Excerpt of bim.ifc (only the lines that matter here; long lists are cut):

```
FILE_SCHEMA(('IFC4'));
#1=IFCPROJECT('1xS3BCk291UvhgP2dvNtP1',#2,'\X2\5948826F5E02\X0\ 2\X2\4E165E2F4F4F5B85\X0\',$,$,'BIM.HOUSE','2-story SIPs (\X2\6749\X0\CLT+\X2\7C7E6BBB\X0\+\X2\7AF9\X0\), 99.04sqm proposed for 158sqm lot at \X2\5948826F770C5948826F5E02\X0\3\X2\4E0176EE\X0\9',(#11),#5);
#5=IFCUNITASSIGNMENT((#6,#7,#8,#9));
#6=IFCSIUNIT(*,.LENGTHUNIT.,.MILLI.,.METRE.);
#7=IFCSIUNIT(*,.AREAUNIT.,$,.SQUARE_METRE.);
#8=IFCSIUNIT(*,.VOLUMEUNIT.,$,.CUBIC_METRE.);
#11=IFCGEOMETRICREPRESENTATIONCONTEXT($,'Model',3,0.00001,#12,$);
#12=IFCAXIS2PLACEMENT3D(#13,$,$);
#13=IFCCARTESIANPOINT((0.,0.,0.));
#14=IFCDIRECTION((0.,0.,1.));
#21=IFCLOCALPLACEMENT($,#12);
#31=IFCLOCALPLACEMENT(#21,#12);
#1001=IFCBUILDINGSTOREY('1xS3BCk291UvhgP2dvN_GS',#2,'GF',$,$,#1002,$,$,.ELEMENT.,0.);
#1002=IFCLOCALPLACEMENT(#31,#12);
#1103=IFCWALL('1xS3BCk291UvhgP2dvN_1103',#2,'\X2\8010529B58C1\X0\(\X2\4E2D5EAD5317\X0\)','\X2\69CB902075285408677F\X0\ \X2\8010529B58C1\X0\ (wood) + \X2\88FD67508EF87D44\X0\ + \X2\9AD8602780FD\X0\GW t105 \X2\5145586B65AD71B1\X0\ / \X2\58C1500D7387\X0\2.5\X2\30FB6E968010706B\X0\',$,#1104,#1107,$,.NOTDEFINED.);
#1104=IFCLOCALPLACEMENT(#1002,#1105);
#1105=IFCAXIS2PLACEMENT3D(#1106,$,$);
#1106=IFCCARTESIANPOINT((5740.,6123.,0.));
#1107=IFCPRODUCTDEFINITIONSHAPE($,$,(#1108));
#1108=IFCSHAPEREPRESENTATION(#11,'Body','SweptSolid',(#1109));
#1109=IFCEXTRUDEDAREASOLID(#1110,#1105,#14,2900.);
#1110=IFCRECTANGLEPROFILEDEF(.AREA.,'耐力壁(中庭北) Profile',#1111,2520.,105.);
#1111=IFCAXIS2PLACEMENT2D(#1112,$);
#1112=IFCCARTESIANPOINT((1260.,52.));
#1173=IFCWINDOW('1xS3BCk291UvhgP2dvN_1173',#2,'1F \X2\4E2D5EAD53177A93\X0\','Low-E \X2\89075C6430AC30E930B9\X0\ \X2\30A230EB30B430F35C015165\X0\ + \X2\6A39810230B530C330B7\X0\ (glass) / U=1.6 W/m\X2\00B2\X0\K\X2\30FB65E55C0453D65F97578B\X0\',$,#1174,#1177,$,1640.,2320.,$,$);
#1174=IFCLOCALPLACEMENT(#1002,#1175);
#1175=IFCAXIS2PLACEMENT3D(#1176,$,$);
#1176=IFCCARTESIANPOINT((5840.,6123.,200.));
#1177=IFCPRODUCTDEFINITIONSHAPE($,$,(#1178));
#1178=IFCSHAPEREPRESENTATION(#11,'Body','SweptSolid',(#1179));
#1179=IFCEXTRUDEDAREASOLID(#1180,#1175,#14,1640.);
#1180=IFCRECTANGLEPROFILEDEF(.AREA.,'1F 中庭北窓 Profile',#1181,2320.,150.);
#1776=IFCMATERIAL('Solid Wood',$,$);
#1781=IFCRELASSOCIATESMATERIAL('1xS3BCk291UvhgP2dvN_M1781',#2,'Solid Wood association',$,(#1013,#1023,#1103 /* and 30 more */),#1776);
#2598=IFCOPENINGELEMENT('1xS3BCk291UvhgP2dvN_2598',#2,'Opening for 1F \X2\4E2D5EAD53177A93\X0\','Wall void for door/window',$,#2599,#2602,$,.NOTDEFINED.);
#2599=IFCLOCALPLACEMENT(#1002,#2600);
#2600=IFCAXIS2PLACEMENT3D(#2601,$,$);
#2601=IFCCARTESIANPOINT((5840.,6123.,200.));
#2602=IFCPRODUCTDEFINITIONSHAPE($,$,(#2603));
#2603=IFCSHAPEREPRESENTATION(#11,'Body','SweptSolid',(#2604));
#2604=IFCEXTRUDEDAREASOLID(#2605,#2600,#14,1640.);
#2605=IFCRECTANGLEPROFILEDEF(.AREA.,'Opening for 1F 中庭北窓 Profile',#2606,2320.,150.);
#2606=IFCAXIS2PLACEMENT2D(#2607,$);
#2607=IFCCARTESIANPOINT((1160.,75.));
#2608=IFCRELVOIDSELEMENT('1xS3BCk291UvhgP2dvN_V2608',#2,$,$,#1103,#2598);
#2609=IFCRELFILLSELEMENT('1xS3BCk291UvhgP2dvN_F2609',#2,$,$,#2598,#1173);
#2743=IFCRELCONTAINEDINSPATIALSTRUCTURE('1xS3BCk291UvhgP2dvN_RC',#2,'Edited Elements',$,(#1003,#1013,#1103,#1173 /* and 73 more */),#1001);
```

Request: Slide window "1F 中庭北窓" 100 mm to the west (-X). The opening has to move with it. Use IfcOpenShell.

```python
import ifcopenshell
import ifcopenshell.api.geometry
import ifcopenshell.util.placement
import ifcopenshell.util.unit

model = ifcopenshell.open("bim.ifc")
unit_scale = ifcopenshell.util.unit.calculate_unit_scale(model)

window = model.by_guid("1xS3BCk291UvhgP2dvN_1173")
opening = window.FillsVoids[0].RelatingOpeningElement
wall = opening.VoidsElements[0].RelatingBuildingElement

wall_matrix = ifcopenshell.util.placement.get_local_placement(wall.ObjectPlacement)
shift = wall_matrix[:3, 0] * -0.1 / unit_scale
before = ifcopenshell.util.placement.get_local_placement(window.ObjectPlacement)[:3, 3].copy()

# The window is not placed relative to its opening, so move both.
for product in (opening, window):
    matrix = ifcopenshell.util.placement.get_local_placement(product.ObjectPlacement)
    matrix[:3, 3] += shift
    ifcopenshell.api.geometry.edit_object_placement(model, product=product, matrix=matrix, is_si=False)

after = ifcopenshell.util.placement.get_local_placement(window.ObjectPlacement)[:3, 3]
print("window moved by", (after - before).round(3) + 0.0)

model.write("bim-out.ifc")
```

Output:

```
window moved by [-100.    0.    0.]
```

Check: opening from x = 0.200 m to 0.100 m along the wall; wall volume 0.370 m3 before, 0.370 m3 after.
